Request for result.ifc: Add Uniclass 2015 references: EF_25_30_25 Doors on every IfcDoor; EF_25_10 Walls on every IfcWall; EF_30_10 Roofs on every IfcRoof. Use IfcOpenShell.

First a look at what the model holds.

```python
import ifcopenshell

model = ifcopenshell.open("result.ifc")
print(model.schema)
print("classifications:", [c.Name for c in model.by_type("IfcClassification")])
for ifc_class in ("IfcDoor", "IfcRoof", "IfcStair", "IfcWall", "IfcWindow"):
    print(ifc_class, len(model.by_type(ifc_class)))
```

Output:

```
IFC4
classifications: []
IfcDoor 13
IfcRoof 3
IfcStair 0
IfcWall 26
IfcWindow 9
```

```python
import ifcopenshell
import ifcopenshell.api.classification

model = ifcopenshell.open("result.ifc")

system = ifcopenshell.api.classification.add_classification(model, classification="Uniclass 2015")

codes = {
    "IfcDoor": ("EF_25_30_25", "Doors"),
    "IfcWall": ("EF_25_10", "Walls"),
    "IfcRoof": ("EF_30_10", "Roofs"),
}
for ifc_class, (code, name) in codes.items():
    products = model.by_type(ifc_class)
    ifcopenshell.api.classification.add_reference(
        model, products=products, classification=system, identification=code, name=name
    )
    print(code, len(products))

model.write("result_edited.ifc")
```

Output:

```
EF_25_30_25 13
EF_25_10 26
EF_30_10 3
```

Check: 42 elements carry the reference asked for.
